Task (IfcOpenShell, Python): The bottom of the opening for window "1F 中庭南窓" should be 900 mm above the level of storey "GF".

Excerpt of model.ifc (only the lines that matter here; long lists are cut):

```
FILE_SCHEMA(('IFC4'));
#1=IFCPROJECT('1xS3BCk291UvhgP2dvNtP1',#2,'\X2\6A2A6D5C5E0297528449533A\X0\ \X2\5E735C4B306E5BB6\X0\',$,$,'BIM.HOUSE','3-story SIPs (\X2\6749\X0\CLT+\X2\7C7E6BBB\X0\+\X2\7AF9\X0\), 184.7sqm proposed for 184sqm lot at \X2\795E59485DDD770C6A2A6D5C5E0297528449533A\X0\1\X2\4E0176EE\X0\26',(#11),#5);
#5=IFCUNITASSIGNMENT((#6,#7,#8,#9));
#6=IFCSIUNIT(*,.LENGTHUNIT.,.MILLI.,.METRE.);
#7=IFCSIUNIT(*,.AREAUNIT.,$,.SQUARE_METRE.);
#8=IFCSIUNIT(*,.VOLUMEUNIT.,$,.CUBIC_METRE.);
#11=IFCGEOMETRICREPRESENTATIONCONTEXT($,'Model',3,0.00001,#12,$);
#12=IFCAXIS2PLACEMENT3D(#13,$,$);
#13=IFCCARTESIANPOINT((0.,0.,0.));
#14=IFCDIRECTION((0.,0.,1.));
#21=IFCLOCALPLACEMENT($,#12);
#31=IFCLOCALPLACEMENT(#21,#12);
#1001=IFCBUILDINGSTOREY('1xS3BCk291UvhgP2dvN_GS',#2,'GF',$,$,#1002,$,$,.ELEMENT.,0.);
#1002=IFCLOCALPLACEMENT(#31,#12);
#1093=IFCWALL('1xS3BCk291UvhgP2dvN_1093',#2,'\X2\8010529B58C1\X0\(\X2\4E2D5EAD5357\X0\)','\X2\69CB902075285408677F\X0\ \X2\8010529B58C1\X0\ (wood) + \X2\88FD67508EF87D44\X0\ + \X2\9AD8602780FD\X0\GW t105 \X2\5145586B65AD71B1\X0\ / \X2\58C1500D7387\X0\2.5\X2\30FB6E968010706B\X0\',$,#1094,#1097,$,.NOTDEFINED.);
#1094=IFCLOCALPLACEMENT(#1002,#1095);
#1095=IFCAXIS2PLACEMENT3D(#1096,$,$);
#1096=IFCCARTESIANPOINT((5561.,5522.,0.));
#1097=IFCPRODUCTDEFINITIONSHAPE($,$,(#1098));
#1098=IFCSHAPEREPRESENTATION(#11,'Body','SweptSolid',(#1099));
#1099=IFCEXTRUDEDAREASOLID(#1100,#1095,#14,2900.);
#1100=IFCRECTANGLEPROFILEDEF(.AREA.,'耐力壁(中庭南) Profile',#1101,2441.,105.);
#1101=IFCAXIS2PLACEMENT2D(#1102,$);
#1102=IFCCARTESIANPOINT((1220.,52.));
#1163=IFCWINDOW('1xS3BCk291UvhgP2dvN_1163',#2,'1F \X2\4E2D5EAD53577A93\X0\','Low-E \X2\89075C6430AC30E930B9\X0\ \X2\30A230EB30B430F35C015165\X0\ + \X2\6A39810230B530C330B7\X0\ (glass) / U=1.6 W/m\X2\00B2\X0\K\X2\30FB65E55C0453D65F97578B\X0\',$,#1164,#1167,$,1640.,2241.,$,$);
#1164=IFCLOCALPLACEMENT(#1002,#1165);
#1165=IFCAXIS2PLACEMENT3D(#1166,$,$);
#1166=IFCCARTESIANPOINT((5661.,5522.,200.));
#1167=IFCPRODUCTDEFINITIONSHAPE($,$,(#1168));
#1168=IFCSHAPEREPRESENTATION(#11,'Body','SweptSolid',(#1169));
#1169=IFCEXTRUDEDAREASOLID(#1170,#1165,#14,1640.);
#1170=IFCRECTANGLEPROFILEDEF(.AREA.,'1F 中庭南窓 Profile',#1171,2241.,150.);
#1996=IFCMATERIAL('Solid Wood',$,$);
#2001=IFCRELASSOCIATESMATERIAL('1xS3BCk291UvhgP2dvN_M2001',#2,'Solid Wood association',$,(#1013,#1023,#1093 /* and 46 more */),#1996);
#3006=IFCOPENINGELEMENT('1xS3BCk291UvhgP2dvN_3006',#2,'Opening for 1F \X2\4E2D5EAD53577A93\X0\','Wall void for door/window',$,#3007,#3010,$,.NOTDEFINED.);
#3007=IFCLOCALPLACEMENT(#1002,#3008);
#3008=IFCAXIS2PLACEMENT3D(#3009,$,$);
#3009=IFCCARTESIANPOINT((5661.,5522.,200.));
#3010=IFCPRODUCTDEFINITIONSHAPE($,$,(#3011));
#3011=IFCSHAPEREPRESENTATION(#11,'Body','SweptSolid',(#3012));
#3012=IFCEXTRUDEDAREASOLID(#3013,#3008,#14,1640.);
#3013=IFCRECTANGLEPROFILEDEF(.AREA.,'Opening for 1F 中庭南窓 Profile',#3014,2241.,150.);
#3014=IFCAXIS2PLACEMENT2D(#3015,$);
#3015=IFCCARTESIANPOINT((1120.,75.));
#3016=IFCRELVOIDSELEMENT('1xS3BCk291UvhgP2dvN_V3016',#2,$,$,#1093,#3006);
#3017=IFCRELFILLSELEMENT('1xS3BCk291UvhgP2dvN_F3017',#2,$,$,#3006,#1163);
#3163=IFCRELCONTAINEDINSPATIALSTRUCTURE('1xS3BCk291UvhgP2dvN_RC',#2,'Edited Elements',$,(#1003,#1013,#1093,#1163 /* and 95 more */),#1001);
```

```python
import numpy as np
import ifcopenshell
import ifcopenshell.api.geometry
import ifcopenshell.geom
import ifcopenshell.util.element
import ifcopenshell.util.placement
import ifcopenshell.util.shape
import ifcopenshell.util.unit

model = ifcopenshell.open("model.ifc")
unit_scale = ifcopenshell.util.unit.calculate_unit_scale(model)

window = model.by_id(1163)
opening = window.FillsVoids[0].RelatingOpeningElement
storey = ifcopenshell.util.element.get_container(window, ifc_class="IfcBuildingStorey")
level = ifcopenshell.util.placement.get_local_placement(storey.ObjectPlacement)[2, 3]

# The opening's origin need not be at the sill, so measure its lowest point.
shape = ifcopenshell.geom.create_shape(ifcopenshell.geom.settings(), opening)
bottom = ifcopenshell.util.shape.get_shape_bottom_elevation(shape, shape.geometry) / unit_scale
dz = level + 0.9 / unit_scale - bottom

shift = np.array([0.0, 0.0, dz])
# The window is not placed relative to its opening, so move both.
for product in (opening, window):
    matrix = ifcopenshell.util.placement.get_local_placement(product.ObjectPlacement)
    matrix[:3, 3] += shift
    ifcopenshell.api.geometry.edit_object_placement(model, product=product, matrix=matrix, is_si=False)

print(f"moved by {dz * unit_scale:+.3f} m")

model.write("model_v2.ifc")
```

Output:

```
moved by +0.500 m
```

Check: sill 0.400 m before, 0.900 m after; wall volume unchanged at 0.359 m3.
